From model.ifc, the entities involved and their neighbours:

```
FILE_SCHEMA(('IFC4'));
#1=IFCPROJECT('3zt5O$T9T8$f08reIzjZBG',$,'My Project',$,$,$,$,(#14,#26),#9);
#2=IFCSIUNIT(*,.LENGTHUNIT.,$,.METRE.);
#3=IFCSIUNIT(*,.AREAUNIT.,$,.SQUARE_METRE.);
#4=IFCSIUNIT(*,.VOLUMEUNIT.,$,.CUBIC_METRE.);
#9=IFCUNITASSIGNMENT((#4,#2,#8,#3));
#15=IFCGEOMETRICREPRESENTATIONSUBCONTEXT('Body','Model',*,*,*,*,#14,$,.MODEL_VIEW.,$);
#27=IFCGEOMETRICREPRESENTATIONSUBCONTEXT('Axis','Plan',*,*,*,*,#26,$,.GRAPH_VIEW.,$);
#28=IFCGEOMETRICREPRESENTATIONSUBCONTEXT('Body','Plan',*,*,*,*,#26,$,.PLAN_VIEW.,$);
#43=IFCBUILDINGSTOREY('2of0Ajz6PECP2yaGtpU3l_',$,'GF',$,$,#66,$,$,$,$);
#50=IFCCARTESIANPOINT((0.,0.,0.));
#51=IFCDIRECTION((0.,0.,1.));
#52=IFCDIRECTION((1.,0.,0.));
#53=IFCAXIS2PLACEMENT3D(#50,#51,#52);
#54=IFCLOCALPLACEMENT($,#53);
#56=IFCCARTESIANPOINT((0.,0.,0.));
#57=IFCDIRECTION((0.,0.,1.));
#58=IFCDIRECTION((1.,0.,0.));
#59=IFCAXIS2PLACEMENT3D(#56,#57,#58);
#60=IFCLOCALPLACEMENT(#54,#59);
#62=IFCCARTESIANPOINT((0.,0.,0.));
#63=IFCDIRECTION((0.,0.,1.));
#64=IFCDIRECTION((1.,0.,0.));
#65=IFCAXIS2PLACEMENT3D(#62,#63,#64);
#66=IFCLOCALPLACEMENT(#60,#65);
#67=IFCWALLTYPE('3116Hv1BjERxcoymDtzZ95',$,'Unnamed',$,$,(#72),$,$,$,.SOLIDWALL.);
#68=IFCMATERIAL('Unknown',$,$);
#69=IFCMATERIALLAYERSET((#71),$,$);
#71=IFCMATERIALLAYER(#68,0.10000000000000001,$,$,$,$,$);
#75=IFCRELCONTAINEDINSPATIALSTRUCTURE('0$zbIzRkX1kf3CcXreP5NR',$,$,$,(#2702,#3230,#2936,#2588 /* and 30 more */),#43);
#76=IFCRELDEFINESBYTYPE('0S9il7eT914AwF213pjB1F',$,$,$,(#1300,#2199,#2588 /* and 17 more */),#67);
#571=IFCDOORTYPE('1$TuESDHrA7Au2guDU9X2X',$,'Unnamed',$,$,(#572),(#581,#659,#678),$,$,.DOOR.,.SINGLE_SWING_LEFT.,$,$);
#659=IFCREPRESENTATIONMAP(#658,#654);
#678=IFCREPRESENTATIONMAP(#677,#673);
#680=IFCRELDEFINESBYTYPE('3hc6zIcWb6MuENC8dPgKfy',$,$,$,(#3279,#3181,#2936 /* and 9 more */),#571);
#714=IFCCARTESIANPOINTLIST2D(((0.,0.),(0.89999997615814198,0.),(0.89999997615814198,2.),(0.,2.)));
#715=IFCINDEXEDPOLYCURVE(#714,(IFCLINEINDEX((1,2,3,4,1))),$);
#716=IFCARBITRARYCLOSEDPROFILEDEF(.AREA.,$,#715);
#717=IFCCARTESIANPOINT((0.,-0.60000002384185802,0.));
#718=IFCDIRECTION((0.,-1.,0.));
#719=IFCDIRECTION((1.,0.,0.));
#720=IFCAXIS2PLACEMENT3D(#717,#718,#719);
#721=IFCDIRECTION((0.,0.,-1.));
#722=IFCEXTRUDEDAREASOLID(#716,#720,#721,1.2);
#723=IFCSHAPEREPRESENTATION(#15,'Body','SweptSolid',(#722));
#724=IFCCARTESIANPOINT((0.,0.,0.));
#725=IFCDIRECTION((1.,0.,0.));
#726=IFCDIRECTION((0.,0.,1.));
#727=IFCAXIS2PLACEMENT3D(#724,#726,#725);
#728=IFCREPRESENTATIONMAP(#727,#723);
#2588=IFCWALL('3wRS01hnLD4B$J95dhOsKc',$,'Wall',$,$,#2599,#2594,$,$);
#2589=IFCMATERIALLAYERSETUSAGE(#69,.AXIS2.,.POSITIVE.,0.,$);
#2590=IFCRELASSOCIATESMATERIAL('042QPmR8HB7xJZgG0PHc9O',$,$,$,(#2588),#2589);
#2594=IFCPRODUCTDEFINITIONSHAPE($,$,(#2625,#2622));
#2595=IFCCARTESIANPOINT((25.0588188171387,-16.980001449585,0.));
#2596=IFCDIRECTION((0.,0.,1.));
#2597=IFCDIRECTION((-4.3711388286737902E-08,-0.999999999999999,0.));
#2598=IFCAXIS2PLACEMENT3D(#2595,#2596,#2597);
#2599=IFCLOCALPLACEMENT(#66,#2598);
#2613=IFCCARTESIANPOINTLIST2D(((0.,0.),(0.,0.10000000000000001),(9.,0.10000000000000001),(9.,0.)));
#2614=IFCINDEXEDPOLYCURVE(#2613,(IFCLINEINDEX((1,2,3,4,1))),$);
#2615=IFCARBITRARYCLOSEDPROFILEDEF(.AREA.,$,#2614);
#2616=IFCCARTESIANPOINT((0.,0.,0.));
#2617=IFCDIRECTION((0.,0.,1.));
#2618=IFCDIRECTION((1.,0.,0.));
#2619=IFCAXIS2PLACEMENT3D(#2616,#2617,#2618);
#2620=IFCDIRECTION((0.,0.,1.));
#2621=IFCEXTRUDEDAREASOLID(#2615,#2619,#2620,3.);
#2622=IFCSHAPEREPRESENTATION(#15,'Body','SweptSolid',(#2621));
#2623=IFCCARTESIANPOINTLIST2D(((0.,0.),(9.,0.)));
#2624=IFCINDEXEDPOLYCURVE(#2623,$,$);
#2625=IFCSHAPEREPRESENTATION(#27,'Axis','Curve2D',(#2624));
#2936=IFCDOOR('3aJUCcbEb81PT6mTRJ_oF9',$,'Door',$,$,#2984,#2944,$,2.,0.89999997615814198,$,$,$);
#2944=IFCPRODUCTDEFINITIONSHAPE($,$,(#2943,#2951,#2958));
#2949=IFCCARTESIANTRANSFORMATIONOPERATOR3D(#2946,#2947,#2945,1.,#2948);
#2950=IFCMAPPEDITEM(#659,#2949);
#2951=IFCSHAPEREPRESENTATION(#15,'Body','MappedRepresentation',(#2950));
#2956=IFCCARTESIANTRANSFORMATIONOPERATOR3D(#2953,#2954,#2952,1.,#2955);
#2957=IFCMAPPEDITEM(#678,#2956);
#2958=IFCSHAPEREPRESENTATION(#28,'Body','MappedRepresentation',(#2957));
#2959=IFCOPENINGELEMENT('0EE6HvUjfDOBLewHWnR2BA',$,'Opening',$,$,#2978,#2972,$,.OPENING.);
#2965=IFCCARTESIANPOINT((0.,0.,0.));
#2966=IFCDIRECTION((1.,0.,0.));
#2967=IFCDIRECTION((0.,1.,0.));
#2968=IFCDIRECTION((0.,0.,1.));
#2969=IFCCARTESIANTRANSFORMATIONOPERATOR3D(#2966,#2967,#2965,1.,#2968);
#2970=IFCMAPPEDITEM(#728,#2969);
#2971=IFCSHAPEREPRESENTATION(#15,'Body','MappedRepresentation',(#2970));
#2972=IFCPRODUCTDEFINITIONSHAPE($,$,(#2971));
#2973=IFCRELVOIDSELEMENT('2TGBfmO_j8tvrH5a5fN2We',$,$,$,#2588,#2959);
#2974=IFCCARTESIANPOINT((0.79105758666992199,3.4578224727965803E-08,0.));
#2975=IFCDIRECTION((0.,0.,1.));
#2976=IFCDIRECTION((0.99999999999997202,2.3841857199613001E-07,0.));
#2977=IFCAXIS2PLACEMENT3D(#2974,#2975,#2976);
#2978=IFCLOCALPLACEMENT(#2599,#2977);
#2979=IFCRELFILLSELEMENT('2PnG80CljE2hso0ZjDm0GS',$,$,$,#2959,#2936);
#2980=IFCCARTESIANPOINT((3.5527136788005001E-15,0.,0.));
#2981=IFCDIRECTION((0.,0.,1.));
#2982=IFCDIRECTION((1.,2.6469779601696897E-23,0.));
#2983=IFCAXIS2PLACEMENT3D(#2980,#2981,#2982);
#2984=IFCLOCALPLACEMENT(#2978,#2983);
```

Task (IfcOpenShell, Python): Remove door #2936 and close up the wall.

```python
import ifcopenshell
import ifcopenshell.api.feature
import ifcopenshell.api.root
import ifcopenshell.geom
import ifcopenshell.util.shape

model = ifcopenshell.open("model.ifc")
settings = ifcopenshell.geom.settings()


def volume(element):
    """Net volume in cubic metres, openings subtracted."""
    shape = ifcopenshell.geom.create_shape(settings, element)
    return ifcopenshell.util.shape.get_volume(shape.geometry)


door = model.by_guid("3aJUCcbEb81PT6mTRJ_oF9")
opening = door.FillsVoids[0].RelatingOpeningElement
wall = opening.VoidsElements[0].RelatingBuildingElement
before = volume(wall)

ifcopenshell.api.root.remove_product(model, product=door)
ifcopenshell.api.feature.remove_feature(model, feature=opening)

after = volume(wall)

print(f"wall volume {before:.3f} -> {after:.3f} m3")

model.write("model-out.ifc")
```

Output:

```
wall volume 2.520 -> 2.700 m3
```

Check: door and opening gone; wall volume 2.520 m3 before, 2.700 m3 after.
